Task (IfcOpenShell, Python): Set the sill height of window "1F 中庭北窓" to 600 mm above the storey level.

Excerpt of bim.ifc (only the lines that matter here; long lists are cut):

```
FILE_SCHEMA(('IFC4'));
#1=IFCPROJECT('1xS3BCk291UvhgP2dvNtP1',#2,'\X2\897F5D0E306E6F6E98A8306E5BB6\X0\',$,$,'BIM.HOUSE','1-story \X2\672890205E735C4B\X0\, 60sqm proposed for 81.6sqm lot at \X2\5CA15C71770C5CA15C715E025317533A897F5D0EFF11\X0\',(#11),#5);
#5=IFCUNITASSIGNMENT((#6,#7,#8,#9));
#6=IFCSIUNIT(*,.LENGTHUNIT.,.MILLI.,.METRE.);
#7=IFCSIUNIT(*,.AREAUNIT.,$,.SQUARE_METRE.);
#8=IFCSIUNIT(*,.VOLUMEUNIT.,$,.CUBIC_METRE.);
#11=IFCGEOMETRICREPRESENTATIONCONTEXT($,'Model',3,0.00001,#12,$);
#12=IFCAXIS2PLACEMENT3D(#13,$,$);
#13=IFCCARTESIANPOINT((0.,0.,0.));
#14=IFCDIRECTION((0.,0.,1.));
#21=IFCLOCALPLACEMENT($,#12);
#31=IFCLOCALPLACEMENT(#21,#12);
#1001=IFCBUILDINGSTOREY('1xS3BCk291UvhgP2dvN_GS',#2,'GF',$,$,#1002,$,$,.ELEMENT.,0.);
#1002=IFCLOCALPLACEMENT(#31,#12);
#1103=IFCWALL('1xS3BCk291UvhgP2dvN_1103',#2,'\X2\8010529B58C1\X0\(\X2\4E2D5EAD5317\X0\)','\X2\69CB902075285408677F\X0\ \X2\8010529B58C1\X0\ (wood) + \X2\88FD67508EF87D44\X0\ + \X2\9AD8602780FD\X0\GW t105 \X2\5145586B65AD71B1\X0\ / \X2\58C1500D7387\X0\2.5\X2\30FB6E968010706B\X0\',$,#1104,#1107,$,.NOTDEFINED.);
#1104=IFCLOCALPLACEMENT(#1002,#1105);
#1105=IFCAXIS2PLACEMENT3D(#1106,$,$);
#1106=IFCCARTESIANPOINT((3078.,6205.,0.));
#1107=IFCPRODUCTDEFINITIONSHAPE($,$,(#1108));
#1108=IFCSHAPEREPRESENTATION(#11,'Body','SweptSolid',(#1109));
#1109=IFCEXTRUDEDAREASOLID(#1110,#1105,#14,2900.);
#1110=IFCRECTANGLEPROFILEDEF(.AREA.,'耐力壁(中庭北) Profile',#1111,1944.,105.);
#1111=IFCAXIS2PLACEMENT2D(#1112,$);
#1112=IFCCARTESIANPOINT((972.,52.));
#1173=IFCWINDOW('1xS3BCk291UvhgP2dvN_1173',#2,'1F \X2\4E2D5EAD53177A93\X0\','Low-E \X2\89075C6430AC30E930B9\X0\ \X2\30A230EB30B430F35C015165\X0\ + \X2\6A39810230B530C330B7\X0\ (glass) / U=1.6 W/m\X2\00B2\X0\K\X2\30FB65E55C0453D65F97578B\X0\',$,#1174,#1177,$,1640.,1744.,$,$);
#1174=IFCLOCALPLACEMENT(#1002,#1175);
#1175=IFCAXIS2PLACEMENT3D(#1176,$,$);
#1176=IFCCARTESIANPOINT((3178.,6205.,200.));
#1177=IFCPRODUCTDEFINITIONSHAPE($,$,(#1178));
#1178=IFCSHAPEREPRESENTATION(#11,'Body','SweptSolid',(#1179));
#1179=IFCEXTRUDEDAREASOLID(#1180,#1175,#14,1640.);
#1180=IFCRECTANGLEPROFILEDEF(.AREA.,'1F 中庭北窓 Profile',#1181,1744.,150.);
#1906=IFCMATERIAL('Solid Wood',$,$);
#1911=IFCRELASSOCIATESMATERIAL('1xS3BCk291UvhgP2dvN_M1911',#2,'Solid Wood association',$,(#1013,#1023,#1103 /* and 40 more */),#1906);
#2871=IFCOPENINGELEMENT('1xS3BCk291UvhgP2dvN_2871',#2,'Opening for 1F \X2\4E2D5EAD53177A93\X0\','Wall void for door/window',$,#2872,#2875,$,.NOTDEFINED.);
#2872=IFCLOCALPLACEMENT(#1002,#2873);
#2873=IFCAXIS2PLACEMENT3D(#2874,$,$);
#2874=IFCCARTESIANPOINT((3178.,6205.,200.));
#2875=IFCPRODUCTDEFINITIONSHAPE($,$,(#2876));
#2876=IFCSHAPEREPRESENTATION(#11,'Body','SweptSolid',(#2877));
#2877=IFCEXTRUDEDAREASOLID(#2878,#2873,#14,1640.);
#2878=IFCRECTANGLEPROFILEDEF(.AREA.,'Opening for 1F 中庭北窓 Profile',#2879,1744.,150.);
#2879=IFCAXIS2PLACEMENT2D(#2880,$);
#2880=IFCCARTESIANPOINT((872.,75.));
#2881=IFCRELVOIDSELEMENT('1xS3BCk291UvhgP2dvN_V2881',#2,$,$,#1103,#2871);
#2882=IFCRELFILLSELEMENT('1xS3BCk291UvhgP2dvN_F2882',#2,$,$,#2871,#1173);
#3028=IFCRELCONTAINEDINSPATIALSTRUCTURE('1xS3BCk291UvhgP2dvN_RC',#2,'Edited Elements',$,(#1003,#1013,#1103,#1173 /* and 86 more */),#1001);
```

```python
import numpy as np
import ifcopenshell
import ifcopenshell.api.geometry
import ifcopenshell.geom
import ifcopenshell.util.element
import ifcopenshell.util.placement
import ifcopenshell.util.shape
import ifcopenshell.util.unit

model = ifcopenshell.open("bim.ifc")
unit_scale = ifcopenshell.util.unit.calculate_unit_scale(model)

window = model.by_guid("1xS3BCk291UvhgP2dvN_1173")
opening = window.FillsVoids[0].RelatingOpeningElement
storey = ifcopenshell.util.element.get_container(window, ifc_class="IfcBuildingStorey")
level = ifcopenshell.util.placement.get_local_placement(storey.ObjectPlacement)[2, 3]

# The opening's origin need not be at the sill, so measure its lowest point.
shape = ifcopenshell.geom.create_shape(ifcopenshell.geom.settings(), opening)
bottom = ifcopenshell.util.shape.get_shape_bottom_elevation(shape, shape.geometry) / unit_scale
dz = level + 0.6 / unit_scale - bottom

shift = np.array([0.0, 0.0, dz])
# The window is not placed relative to its opening, so move both.
for product in (opening, window):
    matrix = ifcopenshell.util.placement.get_local_placement(product.ObjectPlacement)
    matrix[:3, 3] += shift
    ifcopenshell.api.geometry.edit_object_placement(model, product=product, matrix=matrix, is_si=False)

print(f"moved by {dz * unit_scale:+.3f} m")

model.write("bim_edited.ifc")
```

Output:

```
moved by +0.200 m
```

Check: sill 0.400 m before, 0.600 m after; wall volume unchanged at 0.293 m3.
